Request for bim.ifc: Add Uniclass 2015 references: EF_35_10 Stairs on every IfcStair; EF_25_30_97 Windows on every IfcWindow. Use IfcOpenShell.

First a look at what the model holds.

```python
import ifcopenshell

model = ifcopenshell.open("bim.ifc")
print(model.schema)
print("classifications:", [c.Name for c in model.by_type("IfcClassification")])
for ifc_class in ("IfcDoor", "IfcRoof", "IfcStair", "IfcWall", "IfcWindow"):
    print(ifc_class, len(model.by_type(ifc_class)))
```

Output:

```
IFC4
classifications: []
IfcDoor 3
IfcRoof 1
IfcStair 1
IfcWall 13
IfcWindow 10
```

```python
import ifcopenshell
import ifcopenshell.api.classification

model = ifcopenshell.open("bim.ifc")

system = ifcopenshell.api.classification.add_classification(model, classification="Uniclass 2015")

codes = {
    "IfcStair": ("EF_35_10", "Stairs"),
    "IfcWindow": ("EF_25_30_97", "Windows"),
}
for ifc_class, (code, name) in codes.items():
    products = model.by_type(ifc_class)
    ifcopenshell.api.classification.add_reference(
        model, products=products, classification=system, identification=code, name=name
    )
    print(code, len(products))

model.write("bim_edited.ifc")
```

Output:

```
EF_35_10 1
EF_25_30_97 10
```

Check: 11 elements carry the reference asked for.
